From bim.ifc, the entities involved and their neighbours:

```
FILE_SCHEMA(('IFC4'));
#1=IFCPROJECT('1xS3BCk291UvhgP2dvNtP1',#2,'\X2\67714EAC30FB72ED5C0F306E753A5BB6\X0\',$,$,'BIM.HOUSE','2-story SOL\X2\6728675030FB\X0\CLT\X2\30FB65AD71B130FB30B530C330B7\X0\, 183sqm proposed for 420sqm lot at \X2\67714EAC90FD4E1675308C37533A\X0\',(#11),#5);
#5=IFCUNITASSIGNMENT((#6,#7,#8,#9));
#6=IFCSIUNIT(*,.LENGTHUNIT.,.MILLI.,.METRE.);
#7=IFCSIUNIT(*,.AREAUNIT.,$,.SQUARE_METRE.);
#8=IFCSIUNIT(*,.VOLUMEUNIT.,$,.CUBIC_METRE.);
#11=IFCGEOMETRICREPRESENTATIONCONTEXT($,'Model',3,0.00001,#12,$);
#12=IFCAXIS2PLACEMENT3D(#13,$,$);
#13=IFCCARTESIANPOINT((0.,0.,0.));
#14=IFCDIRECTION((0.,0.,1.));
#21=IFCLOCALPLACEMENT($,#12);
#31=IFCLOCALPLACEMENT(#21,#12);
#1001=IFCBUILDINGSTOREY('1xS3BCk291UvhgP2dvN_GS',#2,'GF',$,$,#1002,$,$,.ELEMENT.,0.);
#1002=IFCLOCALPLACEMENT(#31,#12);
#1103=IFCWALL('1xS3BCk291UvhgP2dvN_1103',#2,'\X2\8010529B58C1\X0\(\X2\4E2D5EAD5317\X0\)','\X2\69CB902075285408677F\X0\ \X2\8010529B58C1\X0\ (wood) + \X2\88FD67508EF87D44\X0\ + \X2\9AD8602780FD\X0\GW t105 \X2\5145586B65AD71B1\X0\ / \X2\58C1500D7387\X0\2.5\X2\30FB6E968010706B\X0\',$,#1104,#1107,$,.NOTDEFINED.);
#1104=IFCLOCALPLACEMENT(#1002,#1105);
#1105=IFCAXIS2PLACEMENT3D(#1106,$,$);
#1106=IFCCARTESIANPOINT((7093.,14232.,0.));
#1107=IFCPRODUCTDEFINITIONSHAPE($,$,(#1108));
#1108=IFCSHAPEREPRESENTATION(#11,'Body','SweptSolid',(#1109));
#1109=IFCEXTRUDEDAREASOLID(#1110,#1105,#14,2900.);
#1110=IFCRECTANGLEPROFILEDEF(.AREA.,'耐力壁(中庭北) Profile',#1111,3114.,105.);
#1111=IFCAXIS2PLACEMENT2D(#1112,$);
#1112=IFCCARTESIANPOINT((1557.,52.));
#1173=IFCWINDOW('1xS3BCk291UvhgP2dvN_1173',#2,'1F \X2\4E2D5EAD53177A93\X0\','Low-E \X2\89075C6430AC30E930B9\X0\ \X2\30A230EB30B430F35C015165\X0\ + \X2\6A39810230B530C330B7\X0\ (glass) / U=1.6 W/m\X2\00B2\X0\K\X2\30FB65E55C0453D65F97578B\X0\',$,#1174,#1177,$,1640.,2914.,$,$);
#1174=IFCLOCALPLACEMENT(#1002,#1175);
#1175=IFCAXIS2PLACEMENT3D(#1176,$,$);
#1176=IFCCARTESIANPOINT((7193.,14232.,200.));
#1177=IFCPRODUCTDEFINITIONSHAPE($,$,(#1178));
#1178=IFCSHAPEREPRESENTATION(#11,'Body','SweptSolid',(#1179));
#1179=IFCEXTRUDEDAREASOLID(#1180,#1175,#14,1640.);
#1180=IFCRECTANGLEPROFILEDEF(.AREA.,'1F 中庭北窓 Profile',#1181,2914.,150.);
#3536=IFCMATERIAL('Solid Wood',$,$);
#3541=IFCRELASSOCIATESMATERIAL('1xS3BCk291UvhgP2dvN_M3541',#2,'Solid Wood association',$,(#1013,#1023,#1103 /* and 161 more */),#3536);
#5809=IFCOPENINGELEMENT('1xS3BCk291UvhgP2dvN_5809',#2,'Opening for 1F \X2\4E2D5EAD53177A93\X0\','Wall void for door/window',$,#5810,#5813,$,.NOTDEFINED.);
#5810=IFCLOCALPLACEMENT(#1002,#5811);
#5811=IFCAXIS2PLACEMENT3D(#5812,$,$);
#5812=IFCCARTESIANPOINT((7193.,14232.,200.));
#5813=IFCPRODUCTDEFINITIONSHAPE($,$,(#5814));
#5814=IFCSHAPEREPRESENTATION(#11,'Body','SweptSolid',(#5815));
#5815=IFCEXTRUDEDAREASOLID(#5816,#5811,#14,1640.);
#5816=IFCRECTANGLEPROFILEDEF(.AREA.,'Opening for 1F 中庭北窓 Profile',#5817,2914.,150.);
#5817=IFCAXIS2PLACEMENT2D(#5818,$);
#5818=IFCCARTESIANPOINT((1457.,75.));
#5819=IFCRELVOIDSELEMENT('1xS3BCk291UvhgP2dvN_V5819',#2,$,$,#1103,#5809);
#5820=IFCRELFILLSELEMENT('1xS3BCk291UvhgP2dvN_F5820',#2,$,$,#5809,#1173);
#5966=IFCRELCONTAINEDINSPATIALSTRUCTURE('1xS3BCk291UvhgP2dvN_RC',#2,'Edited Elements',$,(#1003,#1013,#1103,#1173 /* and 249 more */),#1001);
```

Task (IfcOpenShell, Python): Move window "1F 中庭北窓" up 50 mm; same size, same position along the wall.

```python
import numpy as np
import ifcopenshell
import ifcopenshell.api.geometry
import ifcopenshell.util.placement
import ifcopenshell.util.unit

model = ifcopenshell.open("bim.ifc")
unit_scale = ifcopenshell.util.unit.calculate_unit_scale(model)

window = model.by_guid("1xS3BCk291UvhgP2dvN_1173")
opening = window.FillsVoids[0].RelatingOpeningElement
dz = 50.0

shift = np.array([0.0, 0.0, dz])
# The window is not placed relative to its opening, so move both.
for product in (opening, window):
    matrix = ifcopenshell.util.placement.get_local_placement(product.ObjectPlacement)
    matrix[:3, 3] += shift
    ifcopenshell.api.geometry.edit_object_placement(model, product=product, matrix=matrix, is_si=False)

print(f"moved by {dz * unit_scale:+.3f} m")

model.write("bim-out.ifc")
```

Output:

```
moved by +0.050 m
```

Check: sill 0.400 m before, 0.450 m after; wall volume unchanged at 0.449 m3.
